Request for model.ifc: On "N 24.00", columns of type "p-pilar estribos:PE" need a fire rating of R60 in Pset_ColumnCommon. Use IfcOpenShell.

First a look at what the model holds.

```python
import ifcopenshell
import ifcopenshell.util.element

model = ifcopenshell.open("model.ifc")
print(model.schema)
storey = next(s for s in model.by_type("IfcBuildingStorey") if s.Name == "N 24.00")
columns = [e for e in ifcopenshell.util.element.get_decomposition(storey) if e.is_a("IfcColumn")]
seen = {}
for e in columns:
    element_type = ifcopenshell.util.element.get_type(e)
    key = (element_type.Name if element_type != e and element_type else None, ifcopenshell.util.element.get_pset(e, "Pset_ColumnCommon", "FireRating"))
    seen[key] = seen.get(key, 0) + 1
for (name, value), count in sorted(seen.items(), key=str):
    print(count, "x", name, "|", value)
```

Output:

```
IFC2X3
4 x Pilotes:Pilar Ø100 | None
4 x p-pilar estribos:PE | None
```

```python
import ifcopenshell
import ifcopenshell.api.pset
import ifcopenshell.util.element

model = ifcopenshell.open("model.ifc")

storey = next(s for s in model.by_type("IfcBuildingStorey") if s.Name == "N 24.00")
columns = [e for e in ifcopenshell.util.element.get_decomposition(storey) if e.is_a("IfcColumn")]

count = 0
for e in columns:
    element_type = ifcopenshell.util.element.get_type(e)
    if element_type in (None, e) or element_type.Name != "p-pilar estribos:PE":
        continue
    # add_pset returns the element's existing set when there is one.
    pset = ifcopenshell.api.pset.add_pset(model, product=e, name="Pset_ColumnCommon")
    ifcopenshell.api.pset.edit_pset(model, pset=pset, properties={"FireRating": "R60"})
    count += 1

print(count, "columns updated")

model.write("model_edited.ifc")
```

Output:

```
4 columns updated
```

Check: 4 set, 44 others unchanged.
